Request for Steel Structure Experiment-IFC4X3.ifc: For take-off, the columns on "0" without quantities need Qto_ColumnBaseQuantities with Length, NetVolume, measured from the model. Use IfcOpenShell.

First a look at what the model holds.

```python
import ifcopenshell
import ifcopenshell.util.element
import ifcopenshell.util.unit

model = ifcopenshell.open("Steel Structure Experiment-IFC4X3.ifc")
print(model.schema)
for unit_type in ("LENGTHUNIT", "AREAUNIT", "VOLUMEUNIT"):
    print(unit_type, ifcopenshell.util.unit.calculate_unit_scale(model, unit_type))
storey = next(s for s in model.by_type("IfcBuildingStorey") if s.Name == "0")
columns = [e for e in ifcopenshell.util.element.get_decomposition(storey) if e.is_a("IfcColumn")]
for e in sorted(columns, key=lambda e: e.id()):
    print(e.id(), e.is_a(), e.Name, list(ifcopenshell.util.element.get_psets(e, qtos_only=True)), sep=" | ")
```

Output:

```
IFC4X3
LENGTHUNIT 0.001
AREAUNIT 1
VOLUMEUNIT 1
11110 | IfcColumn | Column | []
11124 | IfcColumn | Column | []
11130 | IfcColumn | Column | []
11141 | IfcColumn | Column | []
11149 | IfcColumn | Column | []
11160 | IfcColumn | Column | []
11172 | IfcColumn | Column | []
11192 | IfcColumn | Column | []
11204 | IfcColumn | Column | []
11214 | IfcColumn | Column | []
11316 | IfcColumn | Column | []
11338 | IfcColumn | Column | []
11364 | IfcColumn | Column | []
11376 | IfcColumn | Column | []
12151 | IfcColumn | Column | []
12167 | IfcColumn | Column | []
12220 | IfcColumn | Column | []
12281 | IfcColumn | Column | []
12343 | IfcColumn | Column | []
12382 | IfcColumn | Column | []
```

```python
import ifcopenshell
import ifcopenshell.api.pset
import ifcopenshell.geom
import ifcopenshell.util.element
import ifcopenshell.util.shape
import ifcopenshell.util.unit

model = ifcopenshell.open("Steel Structure Experiment-IFC4X3.ifc")
unit_scale = ifcopenshell.util.unit.calculate_unit_scale(model)
volume_scale = ifcopenshell.util.unit.calculate_unit_scale(model, "VOLUMEUNIT")
settings = ifcopenshell.geom.settings()

storey = next(s for s in model.by_type("IfcBuildingStorey") if s.Name == "0")
columns = [e for e in ifcopenshell.util.element.get_decomposition(storey) if e.is_a("IfcColumn")]

for e in sorted(columns, key=lambda e: e.id()):
    if ifcopenshell.util.element.get_psets(e, qtos_only=True, should_inherit=False):
        continue
    # Geometry comes back in metres, in the element's own axes.
    shape = ifcopenshell.geom.create_shape(settings, e)
    values = {
        "Length": ifcopenshell.util.shape.get_z(shape.geometry) / unit_scale,
        "NetVolume": ifcopenshell.util.shape.get_volume(shape.geometry) / volume_scale,
    }
    qto = ifcopenshell.api.pset.add_qto(model, product=e, name="Qto_ColumnBaseQuantities")
    ifcopenshell.api.pset.edit_qto(model, qto=qto, properties=values)
    print(e.id(), {k: round(v, 3) for k, v in values.items()})

model.write("Steel Structure Experiment-IFC4X3_updated.ifc")
```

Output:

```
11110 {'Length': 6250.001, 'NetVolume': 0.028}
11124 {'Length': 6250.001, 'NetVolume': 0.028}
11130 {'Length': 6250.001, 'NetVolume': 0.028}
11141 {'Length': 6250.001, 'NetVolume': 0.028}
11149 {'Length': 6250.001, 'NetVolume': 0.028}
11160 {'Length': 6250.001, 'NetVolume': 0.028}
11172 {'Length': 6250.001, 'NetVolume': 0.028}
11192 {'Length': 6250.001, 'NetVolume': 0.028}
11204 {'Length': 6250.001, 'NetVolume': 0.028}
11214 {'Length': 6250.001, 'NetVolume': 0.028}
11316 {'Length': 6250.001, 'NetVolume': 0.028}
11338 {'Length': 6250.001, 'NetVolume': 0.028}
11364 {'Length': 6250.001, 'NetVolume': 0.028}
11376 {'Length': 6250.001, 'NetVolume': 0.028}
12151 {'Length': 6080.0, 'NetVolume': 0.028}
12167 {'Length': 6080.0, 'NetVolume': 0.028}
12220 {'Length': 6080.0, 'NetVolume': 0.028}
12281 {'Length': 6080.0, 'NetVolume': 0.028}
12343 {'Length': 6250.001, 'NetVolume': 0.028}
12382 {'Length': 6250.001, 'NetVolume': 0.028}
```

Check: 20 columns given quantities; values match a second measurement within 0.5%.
